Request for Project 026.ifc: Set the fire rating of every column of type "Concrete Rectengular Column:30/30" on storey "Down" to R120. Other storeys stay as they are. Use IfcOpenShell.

First a look at what the model holds.

```python
import ifcopenshell
import ifcopenshell.util.element

model = ifcopenshell.open("Project 026.ifc")
print(model.schema)
storey = next(s for s in model.by_type("IfcBuildingStorey") if s.Name == "Down")
columns = [e for e in ifcopenshell.util.element.get_decomposition(storey) if e.is_a("IfcColumn")]
seen = {}
for e in columns:
    element_type = ifcopenshell.util.element.get_type(e)
    key = (element_type.Name if element_type != e and element_type else None, ifcopenshell.util.element.get_pset(e, "Pset_ColumnCommon", "FireRating"))
    seen[key] = seen.get(key, 0) + 1
for (name, value), count in sorted(seen.items(), key=str):
    print(count, "x", name, "|", value)
```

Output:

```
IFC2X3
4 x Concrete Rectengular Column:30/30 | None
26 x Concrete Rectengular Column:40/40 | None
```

```python
import ifcopenshell
import ifcopenshell.api.pset
import ifcopenshell.util.element

model = ifcopenshell.open("Project 026.ifc")

storey = next(s for s in model.by_type("IfcBuildingStorey") if s.Name == "Down")
columns = [e for e in ifcopenshell.util.element.get_decomposition(storey) if e.is_a("IfcColumn")]

count = 0
for e in columns:
    element_type = ifcopenshell.util.element.get_type(e)
    if element_type in (None, e) or element_type.Name != "Concrete Rectengular Column:30/30":
        continue
    # add_pset returns the element's existing set when there is one.
    pset = ifcopenshell.api.pset.add_pset(model, product=e, name="Pset_ColumnCommon")
    ifcopenshell.api.pset.edit_pset(model, pset=pset, properties={"FireRating": "R120"})
    count += 1

print(count, "columns updated")

model.write("Project 026_rev.ifc")
```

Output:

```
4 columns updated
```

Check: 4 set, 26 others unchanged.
